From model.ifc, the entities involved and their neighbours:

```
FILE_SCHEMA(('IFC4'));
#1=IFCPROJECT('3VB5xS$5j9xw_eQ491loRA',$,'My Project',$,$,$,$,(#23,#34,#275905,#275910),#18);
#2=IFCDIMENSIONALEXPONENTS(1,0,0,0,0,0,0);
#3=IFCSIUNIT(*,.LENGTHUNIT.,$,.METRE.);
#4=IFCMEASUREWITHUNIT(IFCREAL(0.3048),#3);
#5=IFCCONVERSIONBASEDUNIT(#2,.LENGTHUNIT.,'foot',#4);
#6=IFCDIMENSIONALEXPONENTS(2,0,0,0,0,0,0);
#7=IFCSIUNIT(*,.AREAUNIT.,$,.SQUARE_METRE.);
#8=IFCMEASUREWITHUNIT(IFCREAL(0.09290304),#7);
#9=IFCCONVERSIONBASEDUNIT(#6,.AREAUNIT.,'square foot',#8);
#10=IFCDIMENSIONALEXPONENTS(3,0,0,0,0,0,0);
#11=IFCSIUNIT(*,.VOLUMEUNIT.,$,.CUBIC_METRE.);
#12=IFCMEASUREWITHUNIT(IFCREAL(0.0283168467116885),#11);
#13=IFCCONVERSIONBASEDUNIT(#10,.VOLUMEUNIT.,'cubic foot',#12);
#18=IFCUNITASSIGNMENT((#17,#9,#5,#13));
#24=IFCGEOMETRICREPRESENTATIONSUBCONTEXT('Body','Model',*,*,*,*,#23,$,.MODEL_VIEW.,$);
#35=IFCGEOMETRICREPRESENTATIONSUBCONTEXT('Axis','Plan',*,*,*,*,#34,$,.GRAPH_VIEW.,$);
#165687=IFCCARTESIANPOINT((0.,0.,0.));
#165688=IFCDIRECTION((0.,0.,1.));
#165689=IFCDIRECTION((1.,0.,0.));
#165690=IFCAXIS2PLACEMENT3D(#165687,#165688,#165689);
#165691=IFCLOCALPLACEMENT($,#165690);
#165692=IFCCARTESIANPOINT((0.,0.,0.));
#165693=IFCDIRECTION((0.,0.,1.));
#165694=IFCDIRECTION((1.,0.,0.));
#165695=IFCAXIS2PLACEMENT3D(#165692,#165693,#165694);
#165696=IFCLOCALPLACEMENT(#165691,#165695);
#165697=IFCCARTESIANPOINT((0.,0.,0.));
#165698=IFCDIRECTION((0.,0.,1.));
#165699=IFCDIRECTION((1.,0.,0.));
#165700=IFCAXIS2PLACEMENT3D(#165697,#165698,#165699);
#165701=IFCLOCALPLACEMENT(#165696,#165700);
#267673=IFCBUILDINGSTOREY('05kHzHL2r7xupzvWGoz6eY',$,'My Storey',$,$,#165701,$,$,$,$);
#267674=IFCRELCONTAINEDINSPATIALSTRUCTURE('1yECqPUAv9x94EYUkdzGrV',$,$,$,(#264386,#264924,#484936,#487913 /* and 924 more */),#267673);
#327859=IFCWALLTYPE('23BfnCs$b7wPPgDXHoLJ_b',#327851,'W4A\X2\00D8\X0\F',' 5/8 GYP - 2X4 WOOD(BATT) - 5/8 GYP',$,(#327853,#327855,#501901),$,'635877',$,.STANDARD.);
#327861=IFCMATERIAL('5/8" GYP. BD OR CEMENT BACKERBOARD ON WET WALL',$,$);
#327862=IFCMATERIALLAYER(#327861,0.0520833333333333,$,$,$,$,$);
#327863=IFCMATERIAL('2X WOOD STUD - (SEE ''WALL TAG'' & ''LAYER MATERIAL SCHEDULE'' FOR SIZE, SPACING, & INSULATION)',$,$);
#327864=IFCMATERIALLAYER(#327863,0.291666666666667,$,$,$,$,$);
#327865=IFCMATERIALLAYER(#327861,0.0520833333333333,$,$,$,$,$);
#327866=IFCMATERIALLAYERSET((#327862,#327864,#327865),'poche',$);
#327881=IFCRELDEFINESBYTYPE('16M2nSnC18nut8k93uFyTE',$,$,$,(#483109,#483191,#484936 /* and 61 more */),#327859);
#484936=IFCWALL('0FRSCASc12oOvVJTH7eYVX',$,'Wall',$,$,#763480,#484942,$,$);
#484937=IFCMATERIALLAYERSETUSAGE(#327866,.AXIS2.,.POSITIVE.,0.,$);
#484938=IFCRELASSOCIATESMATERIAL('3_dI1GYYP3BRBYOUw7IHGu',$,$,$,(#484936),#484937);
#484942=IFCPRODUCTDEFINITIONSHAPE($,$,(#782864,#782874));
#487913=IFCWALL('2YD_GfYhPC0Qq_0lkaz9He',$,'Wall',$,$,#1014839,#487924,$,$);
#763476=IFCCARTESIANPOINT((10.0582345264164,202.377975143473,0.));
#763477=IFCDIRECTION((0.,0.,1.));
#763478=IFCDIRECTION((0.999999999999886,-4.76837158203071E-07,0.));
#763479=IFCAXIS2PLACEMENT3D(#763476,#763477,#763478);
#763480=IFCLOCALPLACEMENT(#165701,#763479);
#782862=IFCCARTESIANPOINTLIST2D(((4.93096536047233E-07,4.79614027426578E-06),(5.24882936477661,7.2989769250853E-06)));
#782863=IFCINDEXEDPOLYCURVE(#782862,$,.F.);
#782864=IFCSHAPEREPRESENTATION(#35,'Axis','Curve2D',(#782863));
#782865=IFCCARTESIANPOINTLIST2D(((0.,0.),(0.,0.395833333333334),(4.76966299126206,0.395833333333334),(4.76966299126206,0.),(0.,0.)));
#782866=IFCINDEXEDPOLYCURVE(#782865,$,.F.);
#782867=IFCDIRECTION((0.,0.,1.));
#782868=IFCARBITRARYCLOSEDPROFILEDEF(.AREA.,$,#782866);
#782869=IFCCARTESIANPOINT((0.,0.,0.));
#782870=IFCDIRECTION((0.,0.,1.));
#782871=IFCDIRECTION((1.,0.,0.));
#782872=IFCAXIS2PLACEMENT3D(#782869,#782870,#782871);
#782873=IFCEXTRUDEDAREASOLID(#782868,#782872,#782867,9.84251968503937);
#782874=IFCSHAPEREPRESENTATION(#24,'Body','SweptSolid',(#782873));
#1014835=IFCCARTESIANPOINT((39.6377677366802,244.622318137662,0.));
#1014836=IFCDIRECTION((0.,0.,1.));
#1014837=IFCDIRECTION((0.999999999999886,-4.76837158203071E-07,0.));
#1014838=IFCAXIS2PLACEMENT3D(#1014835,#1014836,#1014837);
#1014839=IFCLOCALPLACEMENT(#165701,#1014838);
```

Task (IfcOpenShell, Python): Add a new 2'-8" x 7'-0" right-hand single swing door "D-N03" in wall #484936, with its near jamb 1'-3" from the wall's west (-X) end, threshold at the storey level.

```python
import numpy as np
import ifcopenshell
import ifcopenshell.api.feature
import ifcopenshell.api.geometry
import ifcopenshell.api.root
import ifcopenshell.api.spatial
import ifcopenshell.geom
import ifcopenshell.util.element
import ifcopenshell.util.placement
import ifcopenshell.util.representation
import ifcopenshell.util.shape
import ifcopenshell.util.unit

model = ifcopenshell.open("model.ifc")
unit_scale = ifcopenshell.util.unit.calculate_unit_scale(model)
settings = ifcopenshell.geom.settings()


def volume(element):
    """Net volume in cubic metres, openings subtracted."""
    shape = ifcopenshell.geom.create_shape(settings, element)
    return ifcopenshell.util.shape.get_volume(shape.geometry)


wall = model.by_guid("0FRSCASc12oOvVJTH7eYVX")
storey = ifcopenshell.util.element.get_container(wall, ifc_class="IfcBuildingStorey")
context = ifcopenshell.util.representation.get_context(model, "Model", "Body", "MODEL_VIEW")
before = volume(wall)

width, height, from_end, sill = 0.8128, 2.1336, 0.381, 0.0  # metres

# The wall runs along its own X axis, and the end named is its -X end.
wall_shape = ifcopenshell.geom.create_shape(settings, wall)
x, y, z = ifcopenshell.util.shape.get_vertices(wall_shape.geometry).T
start = x.min() + from_end
face, thickness = float(y.min()), float(y.max() - y.min())
wall_matrix = ifcopenshell.util.placement.get_local_placement(wall.ObjectPlacement)
level = ifcopenshell.util.placement.get_local_placement(storey.ObjectPlacement)[2, 3]


def in_wall(x, y):
    """Placement at x, y metres in the wall's axes, at sill height."""
    matrix = wall_matrix.copy()
    matrix[:, 3] = wall_matrix @ np.array([x / unit_scale, y / unit_scale, 0.0, 1.0])
    matrix[2, 3] = level + sill / unit_scale
    return matrix


# Opening: a box that overshoots both wall faces by 50 mm.
opening = ifcopenshell.api.root.create_entity(model, ifc_class="IfcOpeningElement", predefined_type="OPENING")
box = ifcopenshell.api.geometry.add_wall_representation(
    model, context=context, length=width, height=height, thickness=thickness + 0.1
)
ifcopenshell.api.geometry.assign_representation(model, product=opening, representation=box)
ifcopenshell.api.geometry.edit_object_placement(model, product=opening, matrix=in_wall(start, face - 0.05), is_si=False)
ifcopenshell.api.feature.add_feature(model, feature=opening, element=wall)

door = ifcopenshell.api.root.create_entity(model, ifc_class="IfcDoor", name="D-N03", predefined_type="DOOR")
door.OverallWidth, door.OverallHeight = width / unit_scale, height / unit_scale
door.OperationType = "SINGLE_SWING_RIGHT"
body = ifcopenshell.api.geometry.add_door_representation(
    model,
    context=context,
    overall_width=door.OverallWidth,
    overall_height=door.OverallHeight,
    operation_type="SINGLE_SWING_RIGHT",
    lining_properties={"LiningDepth": thickness / unit_scale, "ThresholdDepth": thickness / unit_scale},
)
ifcopenshell.api.geometry.assign_representation(model, product=door, representation=body)
ifcopenshell.api.spatial.assign_container(model, products=[door], relating_structure=storey)
ifcopenshell.api.feature.add_filling(model, opening=opening, element=door)

# The lining spans the wall, so the door starts at the wall face.
ifcopenshell.api.geometry.edit_object_placement(model, product=door, matrix=in_wall(start, face), is_si=False)

after = volume(wall)

print(f"wall volume {before:.3f} -> {after:.3f} m3")

model.write("model_rev.ifc")
```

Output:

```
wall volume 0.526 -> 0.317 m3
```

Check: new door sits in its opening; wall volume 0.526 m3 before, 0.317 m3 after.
